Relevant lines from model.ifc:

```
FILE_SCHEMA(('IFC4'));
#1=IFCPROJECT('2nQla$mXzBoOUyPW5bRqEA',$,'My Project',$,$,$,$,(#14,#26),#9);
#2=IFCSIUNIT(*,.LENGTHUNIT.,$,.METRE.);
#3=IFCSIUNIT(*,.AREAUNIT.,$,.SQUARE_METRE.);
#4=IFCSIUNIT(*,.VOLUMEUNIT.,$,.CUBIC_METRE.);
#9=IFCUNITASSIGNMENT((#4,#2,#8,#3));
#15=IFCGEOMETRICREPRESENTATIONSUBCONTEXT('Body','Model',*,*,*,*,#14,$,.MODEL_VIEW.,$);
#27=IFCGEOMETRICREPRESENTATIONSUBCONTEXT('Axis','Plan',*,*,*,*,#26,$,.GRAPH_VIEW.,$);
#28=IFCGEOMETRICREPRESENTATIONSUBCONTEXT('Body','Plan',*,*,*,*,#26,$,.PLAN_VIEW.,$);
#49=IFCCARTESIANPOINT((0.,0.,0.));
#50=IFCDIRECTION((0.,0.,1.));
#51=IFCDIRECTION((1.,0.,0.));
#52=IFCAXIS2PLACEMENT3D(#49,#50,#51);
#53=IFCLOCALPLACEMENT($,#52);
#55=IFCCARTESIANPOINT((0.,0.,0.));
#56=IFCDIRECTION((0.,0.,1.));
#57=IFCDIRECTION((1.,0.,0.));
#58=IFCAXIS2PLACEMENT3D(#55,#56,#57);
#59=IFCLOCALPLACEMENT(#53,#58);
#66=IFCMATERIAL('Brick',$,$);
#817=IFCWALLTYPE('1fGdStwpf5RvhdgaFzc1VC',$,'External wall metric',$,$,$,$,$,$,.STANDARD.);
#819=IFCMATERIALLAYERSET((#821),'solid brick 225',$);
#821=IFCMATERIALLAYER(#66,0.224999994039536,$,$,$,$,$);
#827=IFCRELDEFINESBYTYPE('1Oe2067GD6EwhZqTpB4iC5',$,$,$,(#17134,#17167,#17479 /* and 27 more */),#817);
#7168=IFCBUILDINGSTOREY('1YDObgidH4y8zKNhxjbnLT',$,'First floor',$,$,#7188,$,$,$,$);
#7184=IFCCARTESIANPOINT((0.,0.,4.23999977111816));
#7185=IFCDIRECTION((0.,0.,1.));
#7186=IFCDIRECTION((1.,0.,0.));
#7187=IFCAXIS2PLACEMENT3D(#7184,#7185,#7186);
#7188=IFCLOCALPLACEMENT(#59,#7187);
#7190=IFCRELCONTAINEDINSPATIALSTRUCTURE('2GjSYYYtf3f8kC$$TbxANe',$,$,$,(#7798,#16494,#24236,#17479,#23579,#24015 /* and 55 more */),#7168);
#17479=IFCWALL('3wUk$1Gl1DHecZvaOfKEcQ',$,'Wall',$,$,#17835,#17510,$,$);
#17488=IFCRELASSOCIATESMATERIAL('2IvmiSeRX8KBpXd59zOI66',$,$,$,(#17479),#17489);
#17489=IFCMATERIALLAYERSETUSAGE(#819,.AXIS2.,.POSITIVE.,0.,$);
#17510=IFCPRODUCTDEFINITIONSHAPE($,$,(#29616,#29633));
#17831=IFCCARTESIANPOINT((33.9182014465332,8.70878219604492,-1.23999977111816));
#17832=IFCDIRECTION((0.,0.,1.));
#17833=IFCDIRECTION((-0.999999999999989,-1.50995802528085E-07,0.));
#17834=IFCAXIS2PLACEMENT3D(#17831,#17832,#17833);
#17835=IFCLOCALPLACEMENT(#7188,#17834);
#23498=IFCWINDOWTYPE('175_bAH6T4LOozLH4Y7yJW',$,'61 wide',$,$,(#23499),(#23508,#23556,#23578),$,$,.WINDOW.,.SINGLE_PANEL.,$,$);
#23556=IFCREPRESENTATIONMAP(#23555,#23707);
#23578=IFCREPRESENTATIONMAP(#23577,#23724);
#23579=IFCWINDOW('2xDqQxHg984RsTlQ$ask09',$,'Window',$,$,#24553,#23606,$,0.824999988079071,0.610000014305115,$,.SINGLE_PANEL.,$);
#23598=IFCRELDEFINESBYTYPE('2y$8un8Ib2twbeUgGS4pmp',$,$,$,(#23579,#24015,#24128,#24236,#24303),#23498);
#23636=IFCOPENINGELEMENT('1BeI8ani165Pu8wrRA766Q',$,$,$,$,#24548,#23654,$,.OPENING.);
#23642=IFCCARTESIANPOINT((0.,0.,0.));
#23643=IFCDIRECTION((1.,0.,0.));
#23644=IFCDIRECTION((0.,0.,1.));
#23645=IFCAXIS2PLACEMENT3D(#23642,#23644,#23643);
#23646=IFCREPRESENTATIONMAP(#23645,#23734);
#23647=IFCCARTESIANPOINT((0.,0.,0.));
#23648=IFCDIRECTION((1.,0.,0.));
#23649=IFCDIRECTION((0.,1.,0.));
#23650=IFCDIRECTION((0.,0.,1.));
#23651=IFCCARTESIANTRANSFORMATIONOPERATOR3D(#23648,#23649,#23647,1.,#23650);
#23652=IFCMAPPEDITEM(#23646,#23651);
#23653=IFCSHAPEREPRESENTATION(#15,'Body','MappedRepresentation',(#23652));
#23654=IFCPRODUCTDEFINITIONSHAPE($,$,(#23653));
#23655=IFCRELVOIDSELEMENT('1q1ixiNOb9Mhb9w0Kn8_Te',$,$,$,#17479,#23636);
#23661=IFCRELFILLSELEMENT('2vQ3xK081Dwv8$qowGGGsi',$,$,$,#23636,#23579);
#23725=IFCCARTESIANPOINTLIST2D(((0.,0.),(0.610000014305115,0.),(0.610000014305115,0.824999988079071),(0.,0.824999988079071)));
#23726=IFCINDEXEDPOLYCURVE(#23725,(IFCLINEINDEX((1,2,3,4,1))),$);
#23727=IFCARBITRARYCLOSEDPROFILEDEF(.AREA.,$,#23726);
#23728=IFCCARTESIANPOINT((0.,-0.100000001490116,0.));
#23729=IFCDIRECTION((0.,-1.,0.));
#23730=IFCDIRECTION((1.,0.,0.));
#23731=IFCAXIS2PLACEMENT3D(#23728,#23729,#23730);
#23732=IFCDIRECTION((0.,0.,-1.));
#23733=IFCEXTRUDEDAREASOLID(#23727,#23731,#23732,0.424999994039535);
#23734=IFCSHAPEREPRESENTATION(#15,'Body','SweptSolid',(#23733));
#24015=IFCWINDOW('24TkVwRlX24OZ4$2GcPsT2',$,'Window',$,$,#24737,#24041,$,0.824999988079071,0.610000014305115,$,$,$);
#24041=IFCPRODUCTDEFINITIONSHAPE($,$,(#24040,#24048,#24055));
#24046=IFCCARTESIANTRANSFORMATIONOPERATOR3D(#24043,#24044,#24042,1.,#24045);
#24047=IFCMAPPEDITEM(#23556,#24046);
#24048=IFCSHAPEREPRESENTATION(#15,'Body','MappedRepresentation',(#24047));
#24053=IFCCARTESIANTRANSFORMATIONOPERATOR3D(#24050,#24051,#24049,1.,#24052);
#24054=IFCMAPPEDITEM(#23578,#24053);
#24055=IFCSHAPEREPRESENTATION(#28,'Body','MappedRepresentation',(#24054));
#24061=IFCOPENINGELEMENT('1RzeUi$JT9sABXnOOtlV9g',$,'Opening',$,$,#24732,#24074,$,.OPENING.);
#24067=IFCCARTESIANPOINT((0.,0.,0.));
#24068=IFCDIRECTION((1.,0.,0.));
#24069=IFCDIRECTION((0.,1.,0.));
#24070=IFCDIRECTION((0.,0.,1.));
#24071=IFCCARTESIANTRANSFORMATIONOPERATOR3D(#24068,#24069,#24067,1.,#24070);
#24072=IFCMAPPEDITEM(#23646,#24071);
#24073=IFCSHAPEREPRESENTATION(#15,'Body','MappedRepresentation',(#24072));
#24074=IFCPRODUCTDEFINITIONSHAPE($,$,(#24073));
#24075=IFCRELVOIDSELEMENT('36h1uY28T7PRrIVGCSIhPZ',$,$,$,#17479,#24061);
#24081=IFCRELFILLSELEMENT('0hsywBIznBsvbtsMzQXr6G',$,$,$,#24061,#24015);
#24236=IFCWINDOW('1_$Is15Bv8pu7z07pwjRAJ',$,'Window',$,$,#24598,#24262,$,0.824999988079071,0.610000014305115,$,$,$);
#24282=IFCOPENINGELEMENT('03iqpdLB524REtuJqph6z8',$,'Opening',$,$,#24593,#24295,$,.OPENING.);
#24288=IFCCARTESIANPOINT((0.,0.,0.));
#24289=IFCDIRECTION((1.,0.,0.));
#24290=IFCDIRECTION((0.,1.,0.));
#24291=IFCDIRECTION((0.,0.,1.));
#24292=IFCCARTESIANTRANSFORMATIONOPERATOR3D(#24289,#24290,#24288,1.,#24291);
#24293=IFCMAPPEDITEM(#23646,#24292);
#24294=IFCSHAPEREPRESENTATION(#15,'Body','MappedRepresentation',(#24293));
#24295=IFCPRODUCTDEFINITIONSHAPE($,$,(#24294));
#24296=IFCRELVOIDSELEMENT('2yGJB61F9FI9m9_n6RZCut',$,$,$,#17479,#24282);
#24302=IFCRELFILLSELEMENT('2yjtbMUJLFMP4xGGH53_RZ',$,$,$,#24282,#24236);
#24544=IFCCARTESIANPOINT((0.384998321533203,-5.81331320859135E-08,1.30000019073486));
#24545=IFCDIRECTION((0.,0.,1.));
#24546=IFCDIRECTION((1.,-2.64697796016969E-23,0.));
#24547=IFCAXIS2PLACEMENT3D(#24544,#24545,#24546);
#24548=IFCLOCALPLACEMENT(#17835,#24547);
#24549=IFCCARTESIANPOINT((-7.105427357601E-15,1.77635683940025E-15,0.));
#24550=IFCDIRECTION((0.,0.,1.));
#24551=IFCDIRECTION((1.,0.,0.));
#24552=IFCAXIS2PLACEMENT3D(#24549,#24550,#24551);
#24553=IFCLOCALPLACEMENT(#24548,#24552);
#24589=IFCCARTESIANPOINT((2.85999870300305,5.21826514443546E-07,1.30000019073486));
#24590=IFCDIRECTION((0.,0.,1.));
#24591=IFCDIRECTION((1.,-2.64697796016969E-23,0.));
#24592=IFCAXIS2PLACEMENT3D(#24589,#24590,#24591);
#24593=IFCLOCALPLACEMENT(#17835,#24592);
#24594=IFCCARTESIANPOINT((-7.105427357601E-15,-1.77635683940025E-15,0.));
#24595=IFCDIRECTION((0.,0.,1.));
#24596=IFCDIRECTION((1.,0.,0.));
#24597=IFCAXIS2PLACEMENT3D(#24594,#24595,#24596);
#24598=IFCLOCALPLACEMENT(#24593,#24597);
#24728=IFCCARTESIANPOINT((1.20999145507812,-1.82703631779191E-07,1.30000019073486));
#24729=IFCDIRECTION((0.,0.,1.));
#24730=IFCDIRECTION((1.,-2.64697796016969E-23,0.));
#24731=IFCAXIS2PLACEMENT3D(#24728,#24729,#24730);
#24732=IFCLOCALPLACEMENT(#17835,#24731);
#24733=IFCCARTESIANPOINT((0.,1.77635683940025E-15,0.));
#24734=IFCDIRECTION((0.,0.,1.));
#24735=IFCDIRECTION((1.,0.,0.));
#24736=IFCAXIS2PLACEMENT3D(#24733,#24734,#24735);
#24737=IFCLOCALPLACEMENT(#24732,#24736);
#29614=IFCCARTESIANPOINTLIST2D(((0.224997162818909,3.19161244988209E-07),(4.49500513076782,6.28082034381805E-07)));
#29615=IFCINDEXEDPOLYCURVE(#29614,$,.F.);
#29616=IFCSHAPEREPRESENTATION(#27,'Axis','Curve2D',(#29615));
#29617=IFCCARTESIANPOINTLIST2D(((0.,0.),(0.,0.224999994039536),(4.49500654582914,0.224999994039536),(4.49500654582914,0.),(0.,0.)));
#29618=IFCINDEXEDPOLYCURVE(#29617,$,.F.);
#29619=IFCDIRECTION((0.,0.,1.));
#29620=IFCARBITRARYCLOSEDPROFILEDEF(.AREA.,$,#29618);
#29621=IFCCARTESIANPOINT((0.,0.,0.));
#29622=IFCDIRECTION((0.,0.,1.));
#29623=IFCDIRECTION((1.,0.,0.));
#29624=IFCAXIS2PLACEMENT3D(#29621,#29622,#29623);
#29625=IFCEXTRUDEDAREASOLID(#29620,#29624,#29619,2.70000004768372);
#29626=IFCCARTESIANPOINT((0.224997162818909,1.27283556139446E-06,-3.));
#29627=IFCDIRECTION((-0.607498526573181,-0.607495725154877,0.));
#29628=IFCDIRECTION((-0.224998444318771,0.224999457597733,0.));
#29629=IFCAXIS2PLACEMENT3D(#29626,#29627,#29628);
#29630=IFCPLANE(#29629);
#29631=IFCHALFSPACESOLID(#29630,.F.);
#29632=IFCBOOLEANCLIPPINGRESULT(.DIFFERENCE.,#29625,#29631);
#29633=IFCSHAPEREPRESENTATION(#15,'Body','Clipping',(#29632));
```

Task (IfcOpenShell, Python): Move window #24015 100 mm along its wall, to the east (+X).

```python
import ifcopenshell
import ifcopenshell.api.geometry
import ifcopenshell.util.placement
import ifcopenshell.util.unit

model = ifcopenshell.open("model.ifc")
unit_scale = ifcopenshell.util.unit.calculate_unit_scale(model)

window = model.by_guid("24TkVwRlX24OZ4$2GcPsT2")
opening = window.FillsVoids[0].RelatingOpeningElement
wall = opening.VoidsElements[0].RelatingBuildingElement

wall_matrix = ifcopenshell.util.placement.get_local_placement(wall.ObjectPlacement)
shift = wall_matrix[:3, 0] * -0.1 / unit_scale
before = ifcopenshell.util.placement.get_local_placement(window.ObjectPlacement)[:3, 3].copy()

# The window is placed relative to its opening, so it follows when the opening moves.
matrix = ifcopenshell.util.placement.get_local_placement(opening.ObjectPlacement)
matrix[:3, 3] += shift
ifcopenshell.api.geometry.edit_object_placement(
    model, product=opening, matrix=matrix, is_si=False, should_transform_children=True
)

after = ifcopenshell.util.placement.get_local_placement(window.ObjectPlacement)[:3, 3]
print("window moved by", (after - before).round(3) + 0.0)

model.write("model_v2.ifc")
```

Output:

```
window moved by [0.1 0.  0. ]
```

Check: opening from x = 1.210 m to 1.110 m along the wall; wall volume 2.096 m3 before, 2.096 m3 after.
